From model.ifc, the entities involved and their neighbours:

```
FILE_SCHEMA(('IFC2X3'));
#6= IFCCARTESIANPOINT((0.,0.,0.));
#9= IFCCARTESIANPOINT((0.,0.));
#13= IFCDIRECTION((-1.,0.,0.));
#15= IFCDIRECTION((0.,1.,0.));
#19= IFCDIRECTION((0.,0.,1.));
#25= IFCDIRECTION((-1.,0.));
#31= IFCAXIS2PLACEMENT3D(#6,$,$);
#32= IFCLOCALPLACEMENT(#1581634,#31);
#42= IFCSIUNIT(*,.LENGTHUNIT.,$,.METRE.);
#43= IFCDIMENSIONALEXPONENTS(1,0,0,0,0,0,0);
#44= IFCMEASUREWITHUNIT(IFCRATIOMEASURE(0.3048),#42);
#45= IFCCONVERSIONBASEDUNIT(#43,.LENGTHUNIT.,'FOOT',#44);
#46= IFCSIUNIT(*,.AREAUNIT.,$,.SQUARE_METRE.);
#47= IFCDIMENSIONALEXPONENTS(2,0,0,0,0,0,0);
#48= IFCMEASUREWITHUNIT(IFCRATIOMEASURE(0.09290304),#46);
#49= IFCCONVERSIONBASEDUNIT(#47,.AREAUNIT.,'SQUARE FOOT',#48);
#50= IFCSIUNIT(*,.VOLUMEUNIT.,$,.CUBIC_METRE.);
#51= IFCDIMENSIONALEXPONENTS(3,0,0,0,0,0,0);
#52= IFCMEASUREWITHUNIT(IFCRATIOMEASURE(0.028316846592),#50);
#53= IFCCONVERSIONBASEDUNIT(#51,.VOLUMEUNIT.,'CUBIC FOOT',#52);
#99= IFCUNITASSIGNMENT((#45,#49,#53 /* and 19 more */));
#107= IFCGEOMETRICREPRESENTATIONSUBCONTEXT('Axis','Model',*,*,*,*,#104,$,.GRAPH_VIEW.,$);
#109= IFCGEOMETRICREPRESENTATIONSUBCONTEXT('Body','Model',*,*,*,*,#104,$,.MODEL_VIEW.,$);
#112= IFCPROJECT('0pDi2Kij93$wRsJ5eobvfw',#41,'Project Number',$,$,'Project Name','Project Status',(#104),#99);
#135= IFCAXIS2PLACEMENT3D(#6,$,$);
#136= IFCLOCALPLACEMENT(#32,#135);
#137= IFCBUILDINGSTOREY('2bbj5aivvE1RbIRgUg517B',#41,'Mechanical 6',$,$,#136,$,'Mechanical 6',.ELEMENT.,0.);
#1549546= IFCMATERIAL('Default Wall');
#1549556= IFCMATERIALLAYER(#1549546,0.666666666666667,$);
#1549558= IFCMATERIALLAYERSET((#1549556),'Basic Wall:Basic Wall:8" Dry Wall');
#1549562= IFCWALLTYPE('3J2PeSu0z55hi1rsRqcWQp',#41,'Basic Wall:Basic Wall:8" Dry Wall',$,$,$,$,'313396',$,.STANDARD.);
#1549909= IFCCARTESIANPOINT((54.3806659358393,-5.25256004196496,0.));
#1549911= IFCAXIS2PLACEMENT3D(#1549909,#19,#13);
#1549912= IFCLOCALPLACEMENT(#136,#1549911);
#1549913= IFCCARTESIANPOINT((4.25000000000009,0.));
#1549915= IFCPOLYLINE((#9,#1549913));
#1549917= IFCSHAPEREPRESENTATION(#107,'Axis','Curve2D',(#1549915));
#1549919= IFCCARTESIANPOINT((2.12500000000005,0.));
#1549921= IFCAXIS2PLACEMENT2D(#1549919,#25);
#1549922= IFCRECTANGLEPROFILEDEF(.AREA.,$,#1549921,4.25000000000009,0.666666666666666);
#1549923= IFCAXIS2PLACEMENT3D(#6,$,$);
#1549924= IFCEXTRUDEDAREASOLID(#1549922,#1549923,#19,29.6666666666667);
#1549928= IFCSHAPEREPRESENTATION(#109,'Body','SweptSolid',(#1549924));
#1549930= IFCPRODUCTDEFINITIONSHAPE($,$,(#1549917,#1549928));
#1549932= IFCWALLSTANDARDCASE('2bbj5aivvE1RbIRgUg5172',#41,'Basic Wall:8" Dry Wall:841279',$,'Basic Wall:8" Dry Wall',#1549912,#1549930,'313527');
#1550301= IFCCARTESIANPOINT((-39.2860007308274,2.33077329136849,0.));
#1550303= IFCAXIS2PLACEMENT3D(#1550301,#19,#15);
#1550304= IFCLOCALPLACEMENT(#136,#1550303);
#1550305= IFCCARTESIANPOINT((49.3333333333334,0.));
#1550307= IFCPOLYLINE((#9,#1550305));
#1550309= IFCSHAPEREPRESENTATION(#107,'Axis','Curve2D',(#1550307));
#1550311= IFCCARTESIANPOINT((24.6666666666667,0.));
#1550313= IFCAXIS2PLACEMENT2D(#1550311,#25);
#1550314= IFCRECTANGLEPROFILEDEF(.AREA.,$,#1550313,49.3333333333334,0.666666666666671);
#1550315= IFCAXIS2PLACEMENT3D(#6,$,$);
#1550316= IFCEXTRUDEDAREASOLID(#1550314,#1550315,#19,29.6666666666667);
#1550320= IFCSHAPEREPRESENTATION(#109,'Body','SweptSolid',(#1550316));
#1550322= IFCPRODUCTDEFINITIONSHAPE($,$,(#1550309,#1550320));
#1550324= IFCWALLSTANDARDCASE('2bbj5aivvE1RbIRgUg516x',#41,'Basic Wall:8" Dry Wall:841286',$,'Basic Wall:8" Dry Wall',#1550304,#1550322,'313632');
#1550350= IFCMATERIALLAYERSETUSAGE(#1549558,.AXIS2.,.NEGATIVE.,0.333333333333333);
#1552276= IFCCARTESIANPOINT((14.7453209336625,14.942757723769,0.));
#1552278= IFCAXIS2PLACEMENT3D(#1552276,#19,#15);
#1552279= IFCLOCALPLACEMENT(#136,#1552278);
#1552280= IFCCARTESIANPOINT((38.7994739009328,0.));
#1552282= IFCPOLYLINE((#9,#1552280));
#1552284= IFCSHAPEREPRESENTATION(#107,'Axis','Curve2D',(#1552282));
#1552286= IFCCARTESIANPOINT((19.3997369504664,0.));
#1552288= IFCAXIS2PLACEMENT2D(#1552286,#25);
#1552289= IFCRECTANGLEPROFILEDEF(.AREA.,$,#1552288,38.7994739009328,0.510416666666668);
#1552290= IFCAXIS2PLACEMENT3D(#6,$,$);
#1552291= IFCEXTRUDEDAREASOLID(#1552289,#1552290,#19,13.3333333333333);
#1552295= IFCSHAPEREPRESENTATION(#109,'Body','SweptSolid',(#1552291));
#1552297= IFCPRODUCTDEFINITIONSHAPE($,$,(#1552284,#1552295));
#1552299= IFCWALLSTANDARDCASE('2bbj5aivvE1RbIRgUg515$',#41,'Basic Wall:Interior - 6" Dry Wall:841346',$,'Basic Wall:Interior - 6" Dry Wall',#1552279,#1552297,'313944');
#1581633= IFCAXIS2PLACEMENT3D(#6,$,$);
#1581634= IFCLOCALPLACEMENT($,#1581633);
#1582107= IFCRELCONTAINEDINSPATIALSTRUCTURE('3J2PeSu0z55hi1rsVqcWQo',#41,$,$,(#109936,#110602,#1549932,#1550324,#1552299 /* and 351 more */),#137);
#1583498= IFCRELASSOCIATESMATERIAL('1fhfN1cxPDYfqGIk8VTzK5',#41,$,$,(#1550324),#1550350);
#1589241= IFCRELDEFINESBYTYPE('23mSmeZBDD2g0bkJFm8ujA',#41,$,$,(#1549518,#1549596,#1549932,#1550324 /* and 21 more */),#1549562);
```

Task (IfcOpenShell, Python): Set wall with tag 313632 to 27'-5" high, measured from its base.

```python
import ifcopenshell
import ifcopenshell.geom
import ifcopenshell.util.representation
import ifcopenshell.util.shape
import ifcopenshell.util.unit

model = ifcopenshell.open("model.ifc")
unit_scale = ifcopenshell.util.unit.calculate_unit_scale(model)
settings = ifcopenshell.geom.settings()


def volume(element):
    """Net volume in cubic metres, openings subtracted."""
    shape = ifcopenshell.geom.create_shape(settings, element)
    return ifcopenshell.util.shape.get_volume(shape.geometry)


wall = model.by_id(1550324)
before = volume(wall)

body = ifcopenshell.util.representation.get_representation(wall, "Model", "Body")
solid = body.Items[0]
old_height = solid.Depth
solid.Depth = 329 * 0.0254 / unit_scale
after = volume(wall)

print(f"height {old_height:g} -> {solid.Depth:g}, volume {before:.3f} -> {after:.3f} m3")

model.write("model-out.ifc")
```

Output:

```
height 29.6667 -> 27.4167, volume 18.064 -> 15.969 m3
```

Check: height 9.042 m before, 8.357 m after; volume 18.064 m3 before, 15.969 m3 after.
